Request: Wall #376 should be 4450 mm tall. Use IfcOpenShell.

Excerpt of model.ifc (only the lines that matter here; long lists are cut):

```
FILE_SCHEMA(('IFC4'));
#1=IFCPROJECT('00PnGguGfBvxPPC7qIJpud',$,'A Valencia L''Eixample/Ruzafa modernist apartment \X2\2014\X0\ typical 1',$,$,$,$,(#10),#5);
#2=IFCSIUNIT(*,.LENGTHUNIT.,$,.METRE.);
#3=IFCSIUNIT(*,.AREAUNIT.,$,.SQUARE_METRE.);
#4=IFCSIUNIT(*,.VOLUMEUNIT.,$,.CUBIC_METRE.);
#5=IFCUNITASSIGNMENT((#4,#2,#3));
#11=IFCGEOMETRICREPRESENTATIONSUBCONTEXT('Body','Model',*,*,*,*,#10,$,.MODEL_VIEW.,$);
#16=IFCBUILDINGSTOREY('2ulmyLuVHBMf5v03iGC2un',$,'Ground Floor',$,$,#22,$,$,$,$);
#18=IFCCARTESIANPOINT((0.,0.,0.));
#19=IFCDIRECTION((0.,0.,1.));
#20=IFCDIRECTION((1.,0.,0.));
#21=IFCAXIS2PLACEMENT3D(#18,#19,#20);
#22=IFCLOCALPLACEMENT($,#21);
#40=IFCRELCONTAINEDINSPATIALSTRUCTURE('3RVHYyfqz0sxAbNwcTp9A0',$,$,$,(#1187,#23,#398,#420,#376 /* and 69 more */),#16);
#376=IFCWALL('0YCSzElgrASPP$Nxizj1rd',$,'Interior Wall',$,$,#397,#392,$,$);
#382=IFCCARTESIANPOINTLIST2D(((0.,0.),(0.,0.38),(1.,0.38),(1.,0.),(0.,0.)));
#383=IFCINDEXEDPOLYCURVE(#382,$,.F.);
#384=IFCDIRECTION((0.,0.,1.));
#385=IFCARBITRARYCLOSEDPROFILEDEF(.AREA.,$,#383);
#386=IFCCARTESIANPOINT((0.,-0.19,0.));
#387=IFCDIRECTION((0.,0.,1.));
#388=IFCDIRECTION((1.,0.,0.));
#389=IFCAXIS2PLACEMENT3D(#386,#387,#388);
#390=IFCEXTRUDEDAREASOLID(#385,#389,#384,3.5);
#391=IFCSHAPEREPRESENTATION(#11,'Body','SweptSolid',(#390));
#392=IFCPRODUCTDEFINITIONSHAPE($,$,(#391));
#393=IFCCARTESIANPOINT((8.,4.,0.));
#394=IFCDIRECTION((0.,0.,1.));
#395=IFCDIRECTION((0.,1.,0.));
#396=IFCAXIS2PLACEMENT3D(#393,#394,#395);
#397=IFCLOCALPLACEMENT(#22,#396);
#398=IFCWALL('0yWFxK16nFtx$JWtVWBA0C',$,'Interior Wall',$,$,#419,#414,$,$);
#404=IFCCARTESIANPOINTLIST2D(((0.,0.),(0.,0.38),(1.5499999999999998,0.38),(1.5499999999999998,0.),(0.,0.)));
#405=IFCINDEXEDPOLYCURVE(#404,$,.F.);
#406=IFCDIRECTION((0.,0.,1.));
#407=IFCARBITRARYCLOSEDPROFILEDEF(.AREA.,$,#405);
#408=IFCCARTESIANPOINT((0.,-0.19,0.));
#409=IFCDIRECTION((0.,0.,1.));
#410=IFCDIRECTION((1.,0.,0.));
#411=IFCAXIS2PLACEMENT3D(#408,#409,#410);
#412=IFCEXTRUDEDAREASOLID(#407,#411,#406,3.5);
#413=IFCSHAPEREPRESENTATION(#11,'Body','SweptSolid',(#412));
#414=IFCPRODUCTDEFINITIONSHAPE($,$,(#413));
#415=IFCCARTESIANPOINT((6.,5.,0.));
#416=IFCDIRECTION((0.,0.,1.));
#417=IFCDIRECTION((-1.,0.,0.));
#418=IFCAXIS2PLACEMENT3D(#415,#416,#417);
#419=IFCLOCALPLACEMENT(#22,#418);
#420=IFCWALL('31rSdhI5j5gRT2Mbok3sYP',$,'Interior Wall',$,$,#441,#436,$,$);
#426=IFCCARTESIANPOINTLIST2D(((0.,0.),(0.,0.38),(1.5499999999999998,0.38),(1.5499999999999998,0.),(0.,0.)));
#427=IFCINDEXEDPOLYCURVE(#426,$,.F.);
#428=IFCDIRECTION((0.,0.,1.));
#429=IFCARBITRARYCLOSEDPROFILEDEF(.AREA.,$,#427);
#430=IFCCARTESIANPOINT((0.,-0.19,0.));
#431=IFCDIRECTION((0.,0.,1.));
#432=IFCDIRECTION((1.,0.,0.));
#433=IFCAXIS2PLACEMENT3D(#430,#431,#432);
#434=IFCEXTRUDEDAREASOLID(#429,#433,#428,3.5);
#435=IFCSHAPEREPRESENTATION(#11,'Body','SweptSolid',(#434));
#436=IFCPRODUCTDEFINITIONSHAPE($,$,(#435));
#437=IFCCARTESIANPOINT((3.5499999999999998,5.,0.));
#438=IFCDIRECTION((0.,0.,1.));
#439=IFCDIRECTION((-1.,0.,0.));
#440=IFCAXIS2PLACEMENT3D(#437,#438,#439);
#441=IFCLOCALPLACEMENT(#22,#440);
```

```python
import ifcopenshell
import ifcopenshell.geom
import ifcopenshell.util.representation
import ifcopenshell.util.shape
import ifcopenshell.util.unit

model = ifcopenshell.open("model.ifc")
unit_scale = ifcopenshell.util.unit.calculate_unit_scale(model)
settings = ifcopenshell.geom.settings()


def volume(element):
    """Net volume in cubic metres, openings subtracted."""
    shape = ifcopenshell.geom.create_shape(settings, element)
    return ifcopenshell.util.shape.get_volume(shape.geometry)


wall = model.by_guid("0YCSzElgrASPP$Nxizj1rd")
before = volume(wall)

body = ifcopenshell.util.representation.get_representation(wall, "Model", "Body")
solid = body.Items[0]
old_height = solid.Depth
solid.Depth = 4.45 / unit_scale
after = volume(wall)

print(f"height {old_height:g} -> {solid.Depth:g}, volume {before:.3f} -> {after:.3f} m3")

model.write("model-out.ifc")
```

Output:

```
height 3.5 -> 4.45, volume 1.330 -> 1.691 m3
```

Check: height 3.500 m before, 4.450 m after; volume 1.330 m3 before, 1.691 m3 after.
